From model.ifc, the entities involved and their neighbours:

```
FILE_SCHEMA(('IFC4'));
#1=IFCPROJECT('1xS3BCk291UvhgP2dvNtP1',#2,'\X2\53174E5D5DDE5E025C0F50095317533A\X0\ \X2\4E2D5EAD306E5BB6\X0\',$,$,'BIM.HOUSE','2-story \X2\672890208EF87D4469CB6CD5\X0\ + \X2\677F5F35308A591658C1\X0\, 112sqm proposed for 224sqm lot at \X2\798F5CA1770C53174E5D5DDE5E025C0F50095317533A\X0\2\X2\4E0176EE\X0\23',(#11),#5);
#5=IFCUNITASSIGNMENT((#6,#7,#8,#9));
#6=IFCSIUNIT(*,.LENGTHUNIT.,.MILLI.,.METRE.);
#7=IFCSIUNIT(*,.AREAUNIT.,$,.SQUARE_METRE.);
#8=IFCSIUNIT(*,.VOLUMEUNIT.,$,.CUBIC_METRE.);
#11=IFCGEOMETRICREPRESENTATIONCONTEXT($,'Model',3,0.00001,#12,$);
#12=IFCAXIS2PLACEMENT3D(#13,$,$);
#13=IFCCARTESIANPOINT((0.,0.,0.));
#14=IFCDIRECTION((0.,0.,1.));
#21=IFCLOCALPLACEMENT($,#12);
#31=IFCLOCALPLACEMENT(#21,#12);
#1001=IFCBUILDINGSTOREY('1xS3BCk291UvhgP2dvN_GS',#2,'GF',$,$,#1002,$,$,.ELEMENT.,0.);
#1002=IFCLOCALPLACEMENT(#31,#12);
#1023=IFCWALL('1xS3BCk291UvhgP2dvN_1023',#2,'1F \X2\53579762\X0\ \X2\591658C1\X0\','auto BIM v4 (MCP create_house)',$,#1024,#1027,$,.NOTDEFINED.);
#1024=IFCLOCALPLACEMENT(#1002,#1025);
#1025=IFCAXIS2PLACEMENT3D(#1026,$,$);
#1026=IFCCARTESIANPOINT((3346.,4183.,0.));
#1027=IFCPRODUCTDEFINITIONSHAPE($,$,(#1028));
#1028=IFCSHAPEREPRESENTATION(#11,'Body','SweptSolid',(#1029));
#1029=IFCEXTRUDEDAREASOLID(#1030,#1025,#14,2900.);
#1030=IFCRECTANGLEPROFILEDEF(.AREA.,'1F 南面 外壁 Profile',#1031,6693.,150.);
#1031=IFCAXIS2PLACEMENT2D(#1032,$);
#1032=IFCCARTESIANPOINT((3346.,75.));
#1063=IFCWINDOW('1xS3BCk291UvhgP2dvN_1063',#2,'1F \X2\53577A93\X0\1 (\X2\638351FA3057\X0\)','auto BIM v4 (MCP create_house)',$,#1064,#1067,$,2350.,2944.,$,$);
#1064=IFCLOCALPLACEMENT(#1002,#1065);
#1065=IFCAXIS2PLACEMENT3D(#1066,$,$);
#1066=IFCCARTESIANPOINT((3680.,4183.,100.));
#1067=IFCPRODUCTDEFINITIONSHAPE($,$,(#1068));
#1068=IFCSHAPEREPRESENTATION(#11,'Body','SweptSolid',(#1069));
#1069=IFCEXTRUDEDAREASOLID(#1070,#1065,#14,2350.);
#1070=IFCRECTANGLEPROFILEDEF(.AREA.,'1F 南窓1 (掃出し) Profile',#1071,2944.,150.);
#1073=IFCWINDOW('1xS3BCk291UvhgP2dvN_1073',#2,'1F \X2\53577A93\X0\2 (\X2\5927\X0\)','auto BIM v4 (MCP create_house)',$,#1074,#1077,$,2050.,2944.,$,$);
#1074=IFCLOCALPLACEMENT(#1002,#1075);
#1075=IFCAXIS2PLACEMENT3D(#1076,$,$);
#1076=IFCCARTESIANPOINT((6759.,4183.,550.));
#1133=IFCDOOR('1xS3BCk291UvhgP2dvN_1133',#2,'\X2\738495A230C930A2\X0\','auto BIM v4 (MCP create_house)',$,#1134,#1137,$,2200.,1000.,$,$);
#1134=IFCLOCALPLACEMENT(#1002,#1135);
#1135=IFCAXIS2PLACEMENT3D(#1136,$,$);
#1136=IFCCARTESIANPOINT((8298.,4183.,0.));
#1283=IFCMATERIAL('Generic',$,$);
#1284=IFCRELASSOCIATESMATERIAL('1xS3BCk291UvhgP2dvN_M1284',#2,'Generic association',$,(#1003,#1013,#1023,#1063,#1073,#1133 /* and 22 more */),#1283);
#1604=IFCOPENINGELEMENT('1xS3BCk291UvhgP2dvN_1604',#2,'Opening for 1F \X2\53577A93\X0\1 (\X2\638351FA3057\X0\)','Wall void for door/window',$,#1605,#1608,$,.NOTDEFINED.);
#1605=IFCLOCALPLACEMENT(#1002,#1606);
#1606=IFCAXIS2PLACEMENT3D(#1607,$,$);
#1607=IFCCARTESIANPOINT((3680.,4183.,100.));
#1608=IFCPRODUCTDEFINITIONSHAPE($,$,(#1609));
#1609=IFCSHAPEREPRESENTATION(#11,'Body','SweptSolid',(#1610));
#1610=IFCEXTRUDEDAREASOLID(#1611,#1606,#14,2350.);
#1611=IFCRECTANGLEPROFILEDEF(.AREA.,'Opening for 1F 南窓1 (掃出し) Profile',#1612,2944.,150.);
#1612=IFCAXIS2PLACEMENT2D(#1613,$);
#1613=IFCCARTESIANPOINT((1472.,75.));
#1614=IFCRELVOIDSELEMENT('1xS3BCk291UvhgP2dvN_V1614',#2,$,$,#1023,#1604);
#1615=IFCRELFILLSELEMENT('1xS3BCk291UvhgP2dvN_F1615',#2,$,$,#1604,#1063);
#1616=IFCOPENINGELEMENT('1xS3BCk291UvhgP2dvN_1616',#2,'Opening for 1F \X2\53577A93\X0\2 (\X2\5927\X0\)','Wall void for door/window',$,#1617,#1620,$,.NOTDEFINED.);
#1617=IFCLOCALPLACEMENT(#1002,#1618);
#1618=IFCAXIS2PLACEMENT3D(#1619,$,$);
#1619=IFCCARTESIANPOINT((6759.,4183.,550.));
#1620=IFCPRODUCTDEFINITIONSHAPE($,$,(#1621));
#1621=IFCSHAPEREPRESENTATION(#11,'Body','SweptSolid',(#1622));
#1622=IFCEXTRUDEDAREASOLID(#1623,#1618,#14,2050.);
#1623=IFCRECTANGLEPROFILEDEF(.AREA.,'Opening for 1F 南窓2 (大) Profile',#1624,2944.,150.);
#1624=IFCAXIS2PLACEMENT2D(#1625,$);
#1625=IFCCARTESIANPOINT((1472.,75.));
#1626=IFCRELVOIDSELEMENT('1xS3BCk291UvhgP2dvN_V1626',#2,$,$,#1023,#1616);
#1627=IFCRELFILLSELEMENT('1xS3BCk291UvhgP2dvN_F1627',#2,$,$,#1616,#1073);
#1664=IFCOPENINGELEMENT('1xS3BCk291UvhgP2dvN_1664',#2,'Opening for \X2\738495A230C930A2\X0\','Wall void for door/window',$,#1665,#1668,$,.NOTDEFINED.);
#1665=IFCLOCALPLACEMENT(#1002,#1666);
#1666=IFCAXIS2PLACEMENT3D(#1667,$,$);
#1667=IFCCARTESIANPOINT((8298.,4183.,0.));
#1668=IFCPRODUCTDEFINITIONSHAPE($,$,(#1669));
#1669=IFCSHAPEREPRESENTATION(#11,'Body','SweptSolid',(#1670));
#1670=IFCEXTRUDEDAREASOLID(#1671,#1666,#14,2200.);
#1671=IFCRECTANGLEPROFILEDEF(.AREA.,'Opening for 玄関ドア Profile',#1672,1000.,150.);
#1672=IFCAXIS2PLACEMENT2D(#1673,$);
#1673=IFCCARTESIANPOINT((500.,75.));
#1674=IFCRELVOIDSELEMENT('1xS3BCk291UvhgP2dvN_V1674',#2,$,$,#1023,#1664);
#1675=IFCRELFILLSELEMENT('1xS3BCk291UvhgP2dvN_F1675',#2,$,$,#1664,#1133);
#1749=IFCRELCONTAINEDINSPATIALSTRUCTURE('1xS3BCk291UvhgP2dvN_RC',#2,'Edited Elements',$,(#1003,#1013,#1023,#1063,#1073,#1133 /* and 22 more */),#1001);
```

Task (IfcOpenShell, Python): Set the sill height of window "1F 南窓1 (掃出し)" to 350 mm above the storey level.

```python
import numpy as np
import ifcopenshell
import ifcopenshell.api.geometry
import ifcopenshell.geom
import ifcopenshell.util.element
import ifcopenshell.util.placement
import ifcopenshell.util.shape
import ifcopenshell.util.unit

model = ifcopenshell.open("model.ifc")
unit_scale = ifcopenshell.util.unit.calculate_unit_scale(model)

window = model.by_id(1063)
opening = window.FillsVoids[0].RelatingOpeningElement
storey = ifcopenshell.util.element.get_container(window, ifc_class="IfcBuildingStorey")
level = ifcopenshell.util.placement.get_local_placement(storey.ObjectPlacement)[2, 3]

# The opening's origin need not be at the sill, so measure its lowest point.
shape = ifcopenshell.geom.create_shape(ifcopenshell.geom.settings(), opening)
bottom = ifcopenshell.util.shape.get_shape_bottom_elevation(shape, shape.geometry) / unit_scale
dz = level + 350.0 - bottom

shift = np.array([0.0, 0.0, dz])
# The window is not placed relative to its opening, so move both.
for product in (opening, window):
    matrix = ifcopenshell.util.placement.get_local_placement(product.ObjectPlacement)
    matrix[:3, 3] += shift
    ifcopenshell.api.geometry.edit_object_placement(model, product=product, matrix=matrix, is_si=False)

print(f"moved by {dz * unit_scale:+.3f} m")

model.write("model_v2.ifc")
```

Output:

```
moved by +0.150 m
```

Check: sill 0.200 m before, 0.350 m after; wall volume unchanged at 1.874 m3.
